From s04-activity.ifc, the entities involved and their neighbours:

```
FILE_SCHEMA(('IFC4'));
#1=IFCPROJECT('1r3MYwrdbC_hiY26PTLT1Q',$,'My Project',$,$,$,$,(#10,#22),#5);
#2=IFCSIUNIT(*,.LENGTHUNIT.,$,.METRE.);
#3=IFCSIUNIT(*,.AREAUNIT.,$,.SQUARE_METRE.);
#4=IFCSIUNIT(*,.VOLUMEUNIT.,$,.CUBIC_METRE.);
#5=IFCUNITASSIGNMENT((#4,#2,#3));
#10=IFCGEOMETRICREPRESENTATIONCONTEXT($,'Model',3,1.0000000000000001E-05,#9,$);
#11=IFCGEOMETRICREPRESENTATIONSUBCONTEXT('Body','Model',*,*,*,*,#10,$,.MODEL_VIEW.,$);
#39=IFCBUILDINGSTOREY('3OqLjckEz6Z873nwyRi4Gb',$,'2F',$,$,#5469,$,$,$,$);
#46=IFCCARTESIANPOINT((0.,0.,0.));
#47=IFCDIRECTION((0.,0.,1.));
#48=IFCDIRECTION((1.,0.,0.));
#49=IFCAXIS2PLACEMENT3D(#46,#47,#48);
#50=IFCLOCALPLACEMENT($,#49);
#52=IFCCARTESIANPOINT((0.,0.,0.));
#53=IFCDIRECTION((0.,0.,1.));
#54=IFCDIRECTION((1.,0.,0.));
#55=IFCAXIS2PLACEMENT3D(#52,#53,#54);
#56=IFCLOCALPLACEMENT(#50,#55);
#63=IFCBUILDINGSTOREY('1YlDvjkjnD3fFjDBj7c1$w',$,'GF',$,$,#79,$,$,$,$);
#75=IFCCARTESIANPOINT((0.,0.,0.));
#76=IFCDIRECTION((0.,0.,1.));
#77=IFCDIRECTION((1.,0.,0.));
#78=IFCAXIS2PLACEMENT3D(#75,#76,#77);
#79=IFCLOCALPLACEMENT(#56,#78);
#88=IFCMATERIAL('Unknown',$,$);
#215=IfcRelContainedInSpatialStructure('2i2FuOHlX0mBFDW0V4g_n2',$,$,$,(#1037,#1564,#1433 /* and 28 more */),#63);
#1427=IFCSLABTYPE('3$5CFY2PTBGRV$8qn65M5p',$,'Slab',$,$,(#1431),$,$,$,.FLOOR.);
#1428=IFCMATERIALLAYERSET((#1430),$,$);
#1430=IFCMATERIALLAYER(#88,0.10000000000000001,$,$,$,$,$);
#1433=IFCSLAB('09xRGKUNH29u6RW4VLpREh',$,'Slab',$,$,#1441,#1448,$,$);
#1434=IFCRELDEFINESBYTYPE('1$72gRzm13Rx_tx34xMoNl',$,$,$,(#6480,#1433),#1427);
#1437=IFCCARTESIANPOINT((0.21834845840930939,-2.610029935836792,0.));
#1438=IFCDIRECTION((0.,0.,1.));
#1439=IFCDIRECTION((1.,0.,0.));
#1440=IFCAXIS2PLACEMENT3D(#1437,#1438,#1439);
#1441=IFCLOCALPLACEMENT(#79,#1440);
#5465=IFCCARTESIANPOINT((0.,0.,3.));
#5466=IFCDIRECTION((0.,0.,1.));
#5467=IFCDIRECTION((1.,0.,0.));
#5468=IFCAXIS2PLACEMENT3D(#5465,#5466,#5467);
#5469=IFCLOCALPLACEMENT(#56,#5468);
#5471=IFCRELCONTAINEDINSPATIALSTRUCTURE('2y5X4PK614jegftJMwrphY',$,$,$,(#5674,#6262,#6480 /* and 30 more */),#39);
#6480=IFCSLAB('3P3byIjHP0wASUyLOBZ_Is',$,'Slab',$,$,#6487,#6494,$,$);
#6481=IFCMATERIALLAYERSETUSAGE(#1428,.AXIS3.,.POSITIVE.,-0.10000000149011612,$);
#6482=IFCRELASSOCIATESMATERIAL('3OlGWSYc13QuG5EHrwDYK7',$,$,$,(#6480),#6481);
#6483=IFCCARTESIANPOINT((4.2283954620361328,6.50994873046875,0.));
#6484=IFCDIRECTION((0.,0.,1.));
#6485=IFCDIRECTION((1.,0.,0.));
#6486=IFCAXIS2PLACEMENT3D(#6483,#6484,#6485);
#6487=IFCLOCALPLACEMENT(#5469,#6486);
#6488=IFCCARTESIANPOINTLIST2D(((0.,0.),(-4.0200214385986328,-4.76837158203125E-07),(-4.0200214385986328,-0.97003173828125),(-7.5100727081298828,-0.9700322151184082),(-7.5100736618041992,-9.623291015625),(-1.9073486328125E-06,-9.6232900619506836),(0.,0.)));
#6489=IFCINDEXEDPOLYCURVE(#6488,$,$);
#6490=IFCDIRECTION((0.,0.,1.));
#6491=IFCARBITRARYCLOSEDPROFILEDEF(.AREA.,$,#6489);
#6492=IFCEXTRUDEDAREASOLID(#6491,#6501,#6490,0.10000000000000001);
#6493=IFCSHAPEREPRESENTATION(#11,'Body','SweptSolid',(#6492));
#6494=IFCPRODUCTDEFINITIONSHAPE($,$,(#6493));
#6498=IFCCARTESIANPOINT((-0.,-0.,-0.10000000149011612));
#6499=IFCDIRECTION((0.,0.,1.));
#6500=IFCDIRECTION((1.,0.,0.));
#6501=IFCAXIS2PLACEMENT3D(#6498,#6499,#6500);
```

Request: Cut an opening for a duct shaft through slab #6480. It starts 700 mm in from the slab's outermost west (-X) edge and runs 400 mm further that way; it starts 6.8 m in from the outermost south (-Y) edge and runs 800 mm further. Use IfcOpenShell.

```python
import numpy as np
import ifcopenshell
import ifcopenshell.api.feature
import ifcopenshell.api.geometry
import ifcopenshell.api.root
import ifcopenshell.geom
import ifcopenshell.util.placement
import ifcopenshell.util.representation
import ifcopenshell.util.shape
import ifcopenshell.util.unit

model = ifcopenshell.open("s04-activity.ifc")
unit_scale = ifcopenshell.util.unit.calculate_unit_scale(model)
settings = ifcopenshell.geom.settings()


def volume(element):
    """Net volume in cubic metres, openings subtracted."""
    shape = ifcopenshell.geom.create_shape(settings, element)
    return ifcopenshell.util.shape.get_volume(shape.geometry)


slab = model.by_id(6480)
before = volume(slab)

# Extent in the slab's own axes, in metres. The edges named are its -X and -Y sides.
slab_shape = ifcopenshell.geom.create_shape(settings, slab)
vertices = ifcopenshell.util.shape.get_vertices(slab_shape.geometry)
x_min, y_min, bottom = vertices.min(axis=0)
top = vertices[:, 2].max()

opening = ifcopenshell.api.root.create_entity(model, ifc_class="IfcOpeningElement", name="Duct shaft opening", predefined_type="OPENING")
context = ifcopenshell.util.representation.get_context(model, "Model", "Body", "MODEL_VIEW")
width, depth = 0.4, 0.8
outline = [(0.0, 0.0), (width, 0.0), (width, depth), (0.0, depth), (0.0, 0.0)]
# Overshoot both faces by 50 mm so the cut is clean.
shape = ifcopenshell.api.geometry.add_slab_representation(
    model, context=context, depth=top - bottom + 0.1, polyline=outline
)
ifcopenshell.api.geometry.assign_representation(model, product=opening, representation=shape)

matrix = ifcopenshell.util.placement.get_local_placement(slab.ObjectPlacement)
matrix[:, 3] = matrix @ np.append(np.array([x_min + 0.7, y_min + 6.8, bottom - 0.05]) / unit_scale, 1.0)
ifcopenshell.api.geometry.edit_object_placement(model, product=opening, matrix=matrix, is_si=False)
ifcopenshell.api.feature.add_feature(model, feature=opening, element=slab)

after = volume(slab)

print(f"slab volume {before:.3f} -> {after:.3f} m3")

model.write("s04-activity_v2.ifc")
```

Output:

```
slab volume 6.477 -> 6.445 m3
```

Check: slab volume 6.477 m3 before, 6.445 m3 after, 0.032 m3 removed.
